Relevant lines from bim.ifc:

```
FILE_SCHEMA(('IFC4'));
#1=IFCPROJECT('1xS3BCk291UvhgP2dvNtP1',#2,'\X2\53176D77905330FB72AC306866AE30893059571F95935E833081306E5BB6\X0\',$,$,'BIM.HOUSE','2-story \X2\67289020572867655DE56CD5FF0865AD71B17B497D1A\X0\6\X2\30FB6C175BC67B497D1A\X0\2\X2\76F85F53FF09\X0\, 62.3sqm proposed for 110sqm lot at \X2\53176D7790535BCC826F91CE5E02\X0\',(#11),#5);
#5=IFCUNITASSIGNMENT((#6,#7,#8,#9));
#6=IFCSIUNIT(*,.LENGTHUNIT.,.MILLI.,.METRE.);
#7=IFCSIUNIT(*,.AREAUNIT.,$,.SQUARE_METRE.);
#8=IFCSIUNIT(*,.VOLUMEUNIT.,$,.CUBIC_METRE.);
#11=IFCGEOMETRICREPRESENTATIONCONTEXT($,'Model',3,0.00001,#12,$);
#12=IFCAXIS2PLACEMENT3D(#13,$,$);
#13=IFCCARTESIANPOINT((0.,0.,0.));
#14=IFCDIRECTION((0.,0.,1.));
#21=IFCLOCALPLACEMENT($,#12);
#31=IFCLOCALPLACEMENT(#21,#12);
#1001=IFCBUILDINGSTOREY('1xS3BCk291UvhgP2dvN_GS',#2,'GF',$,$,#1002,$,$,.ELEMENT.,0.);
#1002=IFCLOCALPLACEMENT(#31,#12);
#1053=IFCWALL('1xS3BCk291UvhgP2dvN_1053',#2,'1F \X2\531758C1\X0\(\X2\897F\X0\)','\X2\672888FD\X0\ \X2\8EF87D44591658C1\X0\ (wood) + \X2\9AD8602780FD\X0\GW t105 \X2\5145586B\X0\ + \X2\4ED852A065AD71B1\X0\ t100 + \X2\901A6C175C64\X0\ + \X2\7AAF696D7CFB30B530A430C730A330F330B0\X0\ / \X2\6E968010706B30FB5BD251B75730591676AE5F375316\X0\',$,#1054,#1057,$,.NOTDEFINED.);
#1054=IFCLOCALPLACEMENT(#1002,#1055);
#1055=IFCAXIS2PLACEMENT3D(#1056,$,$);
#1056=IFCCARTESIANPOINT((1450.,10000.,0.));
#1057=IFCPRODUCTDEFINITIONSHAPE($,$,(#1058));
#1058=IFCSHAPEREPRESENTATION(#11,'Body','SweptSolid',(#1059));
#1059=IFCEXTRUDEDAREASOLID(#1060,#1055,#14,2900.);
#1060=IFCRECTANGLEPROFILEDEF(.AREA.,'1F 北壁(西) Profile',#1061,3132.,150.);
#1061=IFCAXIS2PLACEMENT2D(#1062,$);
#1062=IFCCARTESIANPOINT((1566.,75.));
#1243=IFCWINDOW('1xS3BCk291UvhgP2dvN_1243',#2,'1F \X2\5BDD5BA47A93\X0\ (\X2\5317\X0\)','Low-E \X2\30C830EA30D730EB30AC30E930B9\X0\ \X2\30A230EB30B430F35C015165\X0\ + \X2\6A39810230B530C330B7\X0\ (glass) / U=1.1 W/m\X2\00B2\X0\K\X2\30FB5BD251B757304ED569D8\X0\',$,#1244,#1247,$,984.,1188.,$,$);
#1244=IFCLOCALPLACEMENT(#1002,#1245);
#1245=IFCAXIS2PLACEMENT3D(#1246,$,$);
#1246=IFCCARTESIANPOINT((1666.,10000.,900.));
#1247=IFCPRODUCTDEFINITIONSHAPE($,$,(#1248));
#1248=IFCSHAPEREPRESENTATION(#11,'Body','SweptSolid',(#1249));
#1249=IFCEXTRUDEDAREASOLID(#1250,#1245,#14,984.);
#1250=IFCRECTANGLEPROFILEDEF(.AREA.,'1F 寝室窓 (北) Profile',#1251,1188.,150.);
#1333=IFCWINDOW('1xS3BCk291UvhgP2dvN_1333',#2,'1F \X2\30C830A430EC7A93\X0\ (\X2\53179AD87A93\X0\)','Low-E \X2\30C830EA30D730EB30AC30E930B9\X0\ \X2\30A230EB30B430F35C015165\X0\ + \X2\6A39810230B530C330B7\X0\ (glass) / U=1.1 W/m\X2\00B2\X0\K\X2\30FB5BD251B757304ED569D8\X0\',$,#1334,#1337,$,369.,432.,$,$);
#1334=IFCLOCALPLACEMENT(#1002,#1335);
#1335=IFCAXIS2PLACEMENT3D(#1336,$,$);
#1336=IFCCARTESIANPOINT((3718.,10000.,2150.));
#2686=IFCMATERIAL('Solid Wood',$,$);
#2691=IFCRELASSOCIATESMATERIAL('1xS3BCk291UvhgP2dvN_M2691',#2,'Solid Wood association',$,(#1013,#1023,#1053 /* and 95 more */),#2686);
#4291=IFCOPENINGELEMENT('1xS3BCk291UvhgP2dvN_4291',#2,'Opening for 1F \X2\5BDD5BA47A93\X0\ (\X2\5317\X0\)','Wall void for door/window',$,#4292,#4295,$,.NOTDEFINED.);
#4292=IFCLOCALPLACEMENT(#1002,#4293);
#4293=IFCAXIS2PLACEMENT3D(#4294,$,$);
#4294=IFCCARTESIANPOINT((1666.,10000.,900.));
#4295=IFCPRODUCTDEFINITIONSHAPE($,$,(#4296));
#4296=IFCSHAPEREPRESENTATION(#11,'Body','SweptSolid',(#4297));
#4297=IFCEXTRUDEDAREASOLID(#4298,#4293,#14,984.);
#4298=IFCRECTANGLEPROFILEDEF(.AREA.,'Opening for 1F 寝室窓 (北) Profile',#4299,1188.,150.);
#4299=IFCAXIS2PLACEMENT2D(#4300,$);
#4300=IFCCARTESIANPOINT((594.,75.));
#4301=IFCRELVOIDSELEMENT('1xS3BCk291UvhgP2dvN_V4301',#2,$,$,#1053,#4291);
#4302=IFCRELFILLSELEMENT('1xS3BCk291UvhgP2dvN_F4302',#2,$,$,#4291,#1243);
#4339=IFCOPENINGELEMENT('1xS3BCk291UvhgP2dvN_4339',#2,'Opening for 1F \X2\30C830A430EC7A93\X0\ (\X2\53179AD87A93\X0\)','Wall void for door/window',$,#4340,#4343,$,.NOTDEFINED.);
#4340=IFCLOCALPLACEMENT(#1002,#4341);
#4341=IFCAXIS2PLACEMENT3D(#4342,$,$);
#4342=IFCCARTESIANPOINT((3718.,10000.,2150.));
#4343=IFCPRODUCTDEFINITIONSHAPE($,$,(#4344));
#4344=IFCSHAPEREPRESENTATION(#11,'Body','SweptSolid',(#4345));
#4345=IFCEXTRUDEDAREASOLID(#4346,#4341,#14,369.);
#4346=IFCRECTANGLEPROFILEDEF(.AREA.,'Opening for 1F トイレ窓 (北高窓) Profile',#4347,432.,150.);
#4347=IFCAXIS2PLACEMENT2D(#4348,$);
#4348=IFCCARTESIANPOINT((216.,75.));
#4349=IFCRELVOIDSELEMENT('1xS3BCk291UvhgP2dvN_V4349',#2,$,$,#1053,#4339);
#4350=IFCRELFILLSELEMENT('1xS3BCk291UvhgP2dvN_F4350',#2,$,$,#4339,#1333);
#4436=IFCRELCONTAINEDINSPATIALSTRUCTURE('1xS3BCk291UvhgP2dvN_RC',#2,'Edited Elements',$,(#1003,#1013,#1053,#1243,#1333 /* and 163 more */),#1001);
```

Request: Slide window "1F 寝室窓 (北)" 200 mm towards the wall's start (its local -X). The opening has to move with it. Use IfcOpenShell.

```python
import ifcopenshell
import ifcopenshell.api.geometry
import ifcopenshell.util.placement

model = ifcopenshell.open("bim.ifc")

window = model.by_id(1243)
opening = window.FillsVoids[0].RelatingOpeningElement
wall = opening.VoidsElements[0].RelatingBuildingElement

wall_matrix = ifcopenshell.util.placement.get_local_placement(wall.ObjectPlacement)
shift = wall_matrix[:3, 0] * -200.0
before = ifcopenshell.util.placement.get_local_placement(window.ObjectPlacement)[:3, 3].copy()

# The window is not placed relative to its opening, so move both.
for product in (opening, window):
    matrix = ifcopenshell.util.placement.get_local_placement(product.ObjectPlacement)
    matrix[:3, 3] += shift
    ifcopenshell.api.geometry.edit_object_placement(model, product=product, matrix=matrix, is_si=False)

after = ifcopenshell.util.placement.get_local_placement(window.ObjectPlacement)[:3, 3]
print("window moved by", (after - before).round(3) + 0.0)

model.write("bim_rev.ifc")
```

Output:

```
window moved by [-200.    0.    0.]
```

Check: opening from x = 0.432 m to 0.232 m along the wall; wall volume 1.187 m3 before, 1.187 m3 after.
